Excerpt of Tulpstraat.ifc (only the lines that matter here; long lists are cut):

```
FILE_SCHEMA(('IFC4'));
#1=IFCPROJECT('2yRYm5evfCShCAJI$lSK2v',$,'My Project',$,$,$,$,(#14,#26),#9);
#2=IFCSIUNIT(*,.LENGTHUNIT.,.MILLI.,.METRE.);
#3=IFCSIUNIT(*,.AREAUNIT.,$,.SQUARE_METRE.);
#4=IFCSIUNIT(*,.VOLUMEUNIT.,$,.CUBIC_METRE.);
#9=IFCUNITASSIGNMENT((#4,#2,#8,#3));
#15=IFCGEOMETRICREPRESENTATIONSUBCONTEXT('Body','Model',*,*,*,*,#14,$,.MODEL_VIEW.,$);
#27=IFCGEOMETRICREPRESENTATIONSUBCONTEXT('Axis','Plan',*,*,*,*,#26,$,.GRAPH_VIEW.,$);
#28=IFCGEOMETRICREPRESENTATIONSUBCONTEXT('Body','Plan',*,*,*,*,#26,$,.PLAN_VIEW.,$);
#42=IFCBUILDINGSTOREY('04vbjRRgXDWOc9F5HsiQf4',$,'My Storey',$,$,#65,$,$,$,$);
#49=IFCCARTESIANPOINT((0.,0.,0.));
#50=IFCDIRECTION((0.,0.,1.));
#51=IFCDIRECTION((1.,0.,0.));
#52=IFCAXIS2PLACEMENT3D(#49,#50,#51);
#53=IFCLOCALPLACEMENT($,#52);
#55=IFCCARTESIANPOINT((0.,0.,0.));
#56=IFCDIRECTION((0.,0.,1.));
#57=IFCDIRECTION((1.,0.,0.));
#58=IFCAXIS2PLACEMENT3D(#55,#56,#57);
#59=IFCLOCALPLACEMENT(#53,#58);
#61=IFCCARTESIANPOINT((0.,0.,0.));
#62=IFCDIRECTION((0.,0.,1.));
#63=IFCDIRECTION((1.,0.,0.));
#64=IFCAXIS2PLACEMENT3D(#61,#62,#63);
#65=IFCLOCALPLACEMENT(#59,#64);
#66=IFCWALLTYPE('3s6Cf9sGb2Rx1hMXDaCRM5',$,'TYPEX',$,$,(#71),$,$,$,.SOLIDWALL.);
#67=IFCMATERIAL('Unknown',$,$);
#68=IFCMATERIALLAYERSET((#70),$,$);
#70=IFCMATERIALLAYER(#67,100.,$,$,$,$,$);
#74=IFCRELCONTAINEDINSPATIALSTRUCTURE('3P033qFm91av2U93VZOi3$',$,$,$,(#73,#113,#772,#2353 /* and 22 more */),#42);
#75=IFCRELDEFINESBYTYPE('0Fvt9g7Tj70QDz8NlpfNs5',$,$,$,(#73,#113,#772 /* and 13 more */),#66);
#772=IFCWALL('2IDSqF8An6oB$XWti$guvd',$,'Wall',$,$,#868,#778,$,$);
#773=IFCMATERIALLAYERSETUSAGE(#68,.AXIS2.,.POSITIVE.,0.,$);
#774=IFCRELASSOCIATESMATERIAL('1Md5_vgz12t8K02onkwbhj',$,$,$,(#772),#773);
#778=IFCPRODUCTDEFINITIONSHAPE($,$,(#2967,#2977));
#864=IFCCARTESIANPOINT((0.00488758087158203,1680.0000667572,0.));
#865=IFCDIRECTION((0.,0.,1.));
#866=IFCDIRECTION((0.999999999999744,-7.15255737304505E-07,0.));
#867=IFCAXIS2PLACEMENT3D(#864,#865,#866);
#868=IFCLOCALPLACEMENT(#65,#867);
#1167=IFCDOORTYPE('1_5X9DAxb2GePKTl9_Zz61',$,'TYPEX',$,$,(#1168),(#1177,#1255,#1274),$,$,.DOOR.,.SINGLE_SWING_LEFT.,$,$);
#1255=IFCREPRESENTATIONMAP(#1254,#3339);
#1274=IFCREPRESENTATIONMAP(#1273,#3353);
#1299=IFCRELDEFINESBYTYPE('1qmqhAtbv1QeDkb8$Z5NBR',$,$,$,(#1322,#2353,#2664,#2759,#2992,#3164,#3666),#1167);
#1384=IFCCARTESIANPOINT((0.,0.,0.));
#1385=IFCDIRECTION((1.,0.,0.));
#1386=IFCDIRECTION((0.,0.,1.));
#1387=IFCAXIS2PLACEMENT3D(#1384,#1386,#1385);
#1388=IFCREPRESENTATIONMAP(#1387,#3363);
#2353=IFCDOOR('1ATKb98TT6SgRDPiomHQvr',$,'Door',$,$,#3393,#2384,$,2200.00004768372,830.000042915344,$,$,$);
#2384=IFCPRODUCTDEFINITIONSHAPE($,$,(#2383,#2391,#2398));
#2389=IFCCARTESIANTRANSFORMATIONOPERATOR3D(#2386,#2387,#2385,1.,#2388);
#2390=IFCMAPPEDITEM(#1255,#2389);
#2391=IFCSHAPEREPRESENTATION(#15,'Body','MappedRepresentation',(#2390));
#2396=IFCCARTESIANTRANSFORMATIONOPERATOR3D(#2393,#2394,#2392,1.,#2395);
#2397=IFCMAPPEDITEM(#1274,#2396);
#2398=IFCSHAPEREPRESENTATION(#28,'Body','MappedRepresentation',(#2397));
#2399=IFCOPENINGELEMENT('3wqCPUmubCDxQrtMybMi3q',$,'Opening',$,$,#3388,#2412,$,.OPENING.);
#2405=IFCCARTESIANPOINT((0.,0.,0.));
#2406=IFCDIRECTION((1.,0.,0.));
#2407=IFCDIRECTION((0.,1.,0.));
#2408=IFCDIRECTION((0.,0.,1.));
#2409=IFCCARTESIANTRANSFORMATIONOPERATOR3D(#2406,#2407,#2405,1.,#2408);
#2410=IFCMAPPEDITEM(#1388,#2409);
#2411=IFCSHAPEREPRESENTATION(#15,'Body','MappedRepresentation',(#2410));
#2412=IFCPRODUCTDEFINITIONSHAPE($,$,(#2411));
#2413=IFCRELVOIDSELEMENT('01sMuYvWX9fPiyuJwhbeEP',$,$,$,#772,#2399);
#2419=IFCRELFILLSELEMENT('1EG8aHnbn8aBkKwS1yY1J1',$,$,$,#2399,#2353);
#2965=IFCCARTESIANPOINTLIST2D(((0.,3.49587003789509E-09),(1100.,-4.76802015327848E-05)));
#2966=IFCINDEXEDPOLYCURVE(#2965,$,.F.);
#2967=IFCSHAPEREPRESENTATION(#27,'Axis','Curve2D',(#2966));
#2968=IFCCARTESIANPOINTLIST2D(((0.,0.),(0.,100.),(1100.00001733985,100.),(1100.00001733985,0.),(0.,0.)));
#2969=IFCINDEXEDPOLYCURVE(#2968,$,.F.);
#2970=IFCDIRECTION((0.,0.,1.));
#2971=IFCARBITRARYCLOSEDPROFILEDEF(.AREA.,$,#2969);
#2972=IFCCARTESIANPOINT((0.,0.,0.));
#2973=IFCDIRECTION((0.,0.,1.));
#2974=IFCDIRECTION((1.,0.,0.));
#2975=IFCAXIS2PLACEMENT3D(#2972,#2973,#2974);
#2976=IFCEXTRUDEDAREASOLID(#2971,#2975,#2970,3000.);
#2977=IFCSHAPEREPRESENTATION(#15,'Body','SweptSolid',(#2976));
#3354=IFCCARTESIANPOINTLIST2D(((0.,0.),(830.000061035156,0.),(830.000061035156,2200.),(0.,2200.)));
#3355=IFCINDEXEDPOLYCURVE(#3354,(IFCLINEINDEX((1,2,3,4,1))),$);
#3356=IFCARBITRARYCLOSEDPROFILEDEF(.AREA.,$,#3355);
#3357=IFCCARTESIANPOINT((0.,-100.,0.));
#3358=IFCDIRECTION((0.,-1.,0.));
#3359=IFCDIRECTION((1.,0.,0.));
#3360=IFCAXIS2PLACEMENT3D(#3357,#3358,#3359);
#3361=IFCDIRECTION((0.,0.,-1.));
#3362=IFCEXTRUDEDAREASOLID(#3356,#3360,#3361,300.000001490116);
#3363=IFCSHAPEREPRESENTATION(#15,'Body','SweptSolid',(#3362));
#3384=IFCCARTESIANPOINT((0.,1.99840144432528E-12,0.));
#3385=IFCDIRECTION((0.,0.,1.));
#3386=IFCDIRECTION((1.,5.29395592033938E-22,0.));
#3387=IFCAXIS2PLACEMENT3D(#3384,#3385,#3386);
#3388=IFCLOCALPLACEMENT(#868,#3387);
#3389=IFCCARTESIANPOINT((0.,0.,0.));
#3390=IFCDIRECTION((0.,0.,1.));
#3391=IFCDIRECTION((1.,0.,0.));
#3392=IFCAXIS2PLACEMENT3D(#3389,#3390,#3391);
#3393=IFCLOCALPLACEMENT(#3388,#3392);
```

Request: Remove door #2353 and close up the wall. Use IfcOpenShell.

```python
import ifcopenshell
import ifcopenshell.api.feature
import ifcopenshell.api.root
import ifcopenshell.geom
import ifcopenshell.util.shape

model = ifcopenshell.open("Tulpstraat.ifc")
settings = ifcopenshell.geom.settings()


def volume(element):
    """Net volume in cubic metres, openings subtracted."""
    shape = ifcopenshell.geom.create_shape(settings, element)
    return ifcopenshell.util.shape.get_volume(shape.geometry)


door = model.by_id(2353)
opening = door.FillsVoids[0].RelatingOpeningElement
wall = opening.VoidsElements[0].RelatingBuildingElement
before = volume(wall)

ifcopenshell.api.root.remove_product(model, product=door)
ifcopenshell.api.feature.remove_feature(model, feature=opening)

after = volume(wall)

print(f"wall volume {before:.3f} -> {after:.3f} m3")

model.write("Tulpstraat_updated.ifc")
```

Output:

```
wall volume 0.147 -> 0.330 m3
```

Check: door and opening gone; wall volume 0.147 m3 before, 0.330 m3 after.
